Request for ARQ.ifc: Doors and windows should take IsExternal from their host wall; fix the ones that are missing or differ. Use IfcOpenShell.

First a look at what the model holds.

```python
import ifcopenshell
import ifcopenshell.util.element

model = ifcopenshell.open("ARQ.ifc")
print(model.schema)
seen = {}
for e in model.by_type("IfcDoor") + model.by_type("IfcWindow"):
    if not e.FillsVoids:
        continue
    host = e.FillsVoids[0].RelatingOpeningElement.VoidsElements[0].RelatingBuildingElement
    own = ifcopenshell.util.element.get_pset(e, f"Pset_{e.is_a()[3:].removesuffix('StandardCase')}Common", "IsExternal")
    wall = ifcopenshell.util.element.get_pset(host, "Pset_WallCommon", "IsExternal")
    seen[e.is_a(), own, wall] = seen.get((e.is_a(), own, wall), 0) + 1
for (cls, own, wall), count in sorted(seen.items(), key=str):
    print(count, cls, "IsExternal:", own, "| host wall:", wall)
```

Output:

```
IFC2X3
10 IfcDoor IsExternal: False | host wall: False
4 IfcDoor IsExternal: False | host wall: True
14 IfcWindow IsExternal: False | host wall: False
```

```python
import ifcopenshell
import ifcopenshell.api.pset
import ifcopenshell.util.element

model = ifcopenshell.open("ARQ.ifc")

count = 0
for ifc_class, pset_name in (("IfcDoor", "Pset_DoorCommon"), ("IfcWindow", "Pset_WindowCommon")):
    for e in model.by_type(ifc_class):
        if not e.FillsVoids:
            continue
        host = e.FillsVoids[0].RelatingOpeningElement.VoidsElements[0].RelatingBuildingElement
        external = ifcopenshell.util.element.get_pset(host, "Pset_WallCommon", "IsExternal")
        if external is None or ifcopenshell.util.element.get_pset(e, pset_name, "IsExternal") == external:
            continue
        pset = ifcopenshell.api.pset.add_pset(model, product=e, name=pset_name)
        ifcopenshell.api.pset.edit_pset(model, pset=pset, properties={"IsExternal": external})
        count += 1

print(count, "updated")

model.write("ARQ_v2.ifc")
```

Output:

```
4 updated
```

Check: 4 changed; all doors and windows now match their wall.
